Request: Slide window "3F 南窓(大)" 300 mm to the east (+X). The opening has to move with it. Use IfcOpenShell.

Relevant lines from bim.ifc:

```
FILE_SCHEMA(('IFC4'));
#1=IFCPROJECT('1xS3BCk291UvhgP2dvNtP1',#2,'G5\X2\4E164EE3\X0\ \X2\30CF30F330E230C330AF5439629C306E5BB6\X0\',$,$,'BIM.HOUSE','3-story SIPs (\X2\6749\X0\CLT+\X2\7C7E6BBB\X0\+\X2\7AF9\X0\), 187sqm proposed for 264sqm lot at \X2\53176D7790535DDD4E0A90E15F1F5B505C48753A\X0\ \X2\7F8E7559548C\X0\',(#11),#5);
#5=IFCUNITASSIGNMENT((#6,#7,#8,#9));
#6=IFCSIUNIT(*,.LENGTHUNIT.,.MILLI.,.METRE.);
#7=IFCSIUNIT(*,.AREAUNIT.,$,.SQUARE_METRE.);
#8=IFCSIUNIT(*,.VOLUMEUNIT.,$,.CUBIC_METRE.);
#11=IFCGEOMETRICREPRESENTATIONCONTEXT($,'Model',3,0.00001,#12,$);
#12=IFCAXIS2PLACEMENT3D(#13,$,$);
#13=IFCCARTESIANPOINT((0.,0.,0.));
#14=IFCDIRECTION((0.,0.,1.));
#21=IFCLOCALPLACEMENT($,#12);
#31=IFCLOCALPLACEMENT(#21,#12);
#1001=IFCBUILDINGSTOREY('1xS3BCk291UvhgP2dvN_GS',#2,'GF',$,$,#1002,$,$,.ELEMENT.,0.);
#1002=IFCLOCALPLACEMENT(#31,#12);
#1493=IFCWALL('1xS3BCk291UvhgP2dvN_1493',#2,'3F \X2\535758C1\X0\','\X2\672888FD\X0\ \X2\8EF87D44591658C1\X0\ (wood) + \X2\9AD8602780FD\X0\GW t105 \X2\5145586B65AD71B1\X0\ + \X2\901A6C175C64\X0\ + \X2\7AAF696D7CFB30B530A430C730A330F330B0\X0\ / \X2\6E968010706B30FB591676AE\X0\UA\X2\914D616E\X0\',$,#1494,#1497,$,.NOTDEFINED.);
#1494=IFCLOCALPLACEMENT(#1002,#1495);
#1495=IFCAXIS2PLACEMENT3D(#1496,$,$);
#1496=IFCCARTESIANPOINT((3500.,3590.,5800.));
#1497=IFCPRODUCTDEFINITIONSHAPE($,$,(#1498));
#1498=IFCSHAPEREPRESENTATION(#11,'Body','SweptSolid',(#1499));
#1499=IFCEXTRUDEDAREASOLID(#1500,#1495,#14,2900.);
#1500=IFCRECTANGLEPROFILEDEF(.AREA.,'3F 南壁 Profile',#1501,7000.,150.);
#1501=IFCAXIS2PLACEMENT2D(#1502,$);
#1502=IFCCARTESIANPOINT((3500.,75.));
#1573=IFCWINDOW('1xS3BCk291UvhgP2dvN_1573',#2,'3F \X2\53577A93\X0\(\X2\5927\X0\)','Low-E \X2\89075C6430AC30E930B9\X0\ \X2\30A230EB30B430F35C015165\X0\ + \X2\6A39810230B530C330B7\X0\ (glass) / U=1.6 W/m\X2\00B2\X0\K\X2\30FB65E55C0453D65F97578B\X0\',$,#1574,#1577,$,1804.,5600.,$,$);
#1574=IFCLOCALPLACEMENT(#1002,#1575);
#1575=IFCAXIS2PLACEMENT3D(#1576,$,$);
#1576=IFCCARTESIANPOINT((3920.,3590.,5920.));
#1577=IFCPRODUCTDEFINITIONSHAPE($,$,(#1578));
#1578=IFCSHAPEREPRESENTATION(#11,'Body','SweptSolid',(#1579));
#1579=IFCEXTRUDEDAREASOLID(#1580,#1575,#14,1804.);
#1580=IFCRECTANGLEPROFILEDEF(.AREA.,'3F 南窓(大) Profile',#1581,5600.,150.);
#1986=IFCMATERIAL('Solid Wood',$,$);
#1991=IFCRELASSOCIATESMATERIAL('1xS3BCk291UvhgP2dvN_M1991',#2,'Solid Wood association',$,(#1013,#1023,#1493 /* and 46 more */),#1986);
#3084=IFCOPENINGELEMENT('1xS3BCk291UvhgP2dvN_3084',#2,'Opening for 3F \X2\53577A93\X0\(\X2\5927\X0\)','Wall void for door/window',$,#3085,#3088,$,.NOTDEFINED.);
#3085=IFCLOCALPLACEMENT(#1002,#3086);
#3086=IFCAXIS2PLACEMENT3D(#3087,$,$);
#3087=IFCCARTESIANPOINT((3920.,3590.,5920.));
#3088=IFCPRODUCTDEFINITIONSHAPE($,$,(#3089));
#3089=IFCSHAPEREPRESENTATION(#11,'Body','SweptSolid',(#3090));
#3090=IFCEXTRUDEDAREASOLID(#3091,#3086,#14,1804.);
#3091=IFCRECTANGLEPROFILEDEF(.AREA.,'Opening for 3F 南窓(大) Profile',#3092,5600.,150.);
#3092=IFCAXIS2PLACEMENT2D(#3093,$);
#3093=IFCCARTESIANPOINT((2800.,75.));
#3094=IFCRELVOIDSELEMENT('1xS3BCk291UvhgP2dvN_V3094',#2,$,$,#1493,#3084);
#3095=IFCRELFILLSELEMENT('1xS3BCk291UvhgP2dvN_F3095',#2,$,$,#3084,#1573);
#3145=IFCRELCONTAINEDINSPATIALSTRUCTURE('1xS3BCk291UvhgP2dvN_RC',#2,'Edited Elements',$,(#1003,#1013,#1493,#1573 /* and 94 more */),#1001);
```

```python
import ifcopenshell
import ifcopenshell.api.geometry
import ifcopenshell.util.placement

model = ifcopenshell.open("bim.ifc")

window = model.by_id(1573)
opening = window.FillsVoids[0].RelatingOpeningElement
wall = opening.VoidsElements[0].RelatingBuildingElement

wall_matrix = ifcopenshell.util.placement.get_local_placement(wall.ObjectPlacement)
shift = wall_matrix[:3, 0] * 300.0
before = ifcopenshell.util.placement.get_local_placement(window.ObjectPlacement)[:3, 3].copy()

# The window is not placed relative to its opening, so move both.
for product in (opening, window):
    matrix = ifcopenshell.util.placement.get_local_placement(product.ObjectPlacement)
    matrix[:3, 3] += shift
    ifcopenshell.api.geometry.edit_object_placement(model, product=product, matrix=matrix, is_si=False)

after = ifcopenshell.util.placement.get_local_placement(window.ObjectPlacement)[:3, 3]
print("window moved by", (after - before).round(3) + 0.0)

model.write("bim_updated.ifc")
```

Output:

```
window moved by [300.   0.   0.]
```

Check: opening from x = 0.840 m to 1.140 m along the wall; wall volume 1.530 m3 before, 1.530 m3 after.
